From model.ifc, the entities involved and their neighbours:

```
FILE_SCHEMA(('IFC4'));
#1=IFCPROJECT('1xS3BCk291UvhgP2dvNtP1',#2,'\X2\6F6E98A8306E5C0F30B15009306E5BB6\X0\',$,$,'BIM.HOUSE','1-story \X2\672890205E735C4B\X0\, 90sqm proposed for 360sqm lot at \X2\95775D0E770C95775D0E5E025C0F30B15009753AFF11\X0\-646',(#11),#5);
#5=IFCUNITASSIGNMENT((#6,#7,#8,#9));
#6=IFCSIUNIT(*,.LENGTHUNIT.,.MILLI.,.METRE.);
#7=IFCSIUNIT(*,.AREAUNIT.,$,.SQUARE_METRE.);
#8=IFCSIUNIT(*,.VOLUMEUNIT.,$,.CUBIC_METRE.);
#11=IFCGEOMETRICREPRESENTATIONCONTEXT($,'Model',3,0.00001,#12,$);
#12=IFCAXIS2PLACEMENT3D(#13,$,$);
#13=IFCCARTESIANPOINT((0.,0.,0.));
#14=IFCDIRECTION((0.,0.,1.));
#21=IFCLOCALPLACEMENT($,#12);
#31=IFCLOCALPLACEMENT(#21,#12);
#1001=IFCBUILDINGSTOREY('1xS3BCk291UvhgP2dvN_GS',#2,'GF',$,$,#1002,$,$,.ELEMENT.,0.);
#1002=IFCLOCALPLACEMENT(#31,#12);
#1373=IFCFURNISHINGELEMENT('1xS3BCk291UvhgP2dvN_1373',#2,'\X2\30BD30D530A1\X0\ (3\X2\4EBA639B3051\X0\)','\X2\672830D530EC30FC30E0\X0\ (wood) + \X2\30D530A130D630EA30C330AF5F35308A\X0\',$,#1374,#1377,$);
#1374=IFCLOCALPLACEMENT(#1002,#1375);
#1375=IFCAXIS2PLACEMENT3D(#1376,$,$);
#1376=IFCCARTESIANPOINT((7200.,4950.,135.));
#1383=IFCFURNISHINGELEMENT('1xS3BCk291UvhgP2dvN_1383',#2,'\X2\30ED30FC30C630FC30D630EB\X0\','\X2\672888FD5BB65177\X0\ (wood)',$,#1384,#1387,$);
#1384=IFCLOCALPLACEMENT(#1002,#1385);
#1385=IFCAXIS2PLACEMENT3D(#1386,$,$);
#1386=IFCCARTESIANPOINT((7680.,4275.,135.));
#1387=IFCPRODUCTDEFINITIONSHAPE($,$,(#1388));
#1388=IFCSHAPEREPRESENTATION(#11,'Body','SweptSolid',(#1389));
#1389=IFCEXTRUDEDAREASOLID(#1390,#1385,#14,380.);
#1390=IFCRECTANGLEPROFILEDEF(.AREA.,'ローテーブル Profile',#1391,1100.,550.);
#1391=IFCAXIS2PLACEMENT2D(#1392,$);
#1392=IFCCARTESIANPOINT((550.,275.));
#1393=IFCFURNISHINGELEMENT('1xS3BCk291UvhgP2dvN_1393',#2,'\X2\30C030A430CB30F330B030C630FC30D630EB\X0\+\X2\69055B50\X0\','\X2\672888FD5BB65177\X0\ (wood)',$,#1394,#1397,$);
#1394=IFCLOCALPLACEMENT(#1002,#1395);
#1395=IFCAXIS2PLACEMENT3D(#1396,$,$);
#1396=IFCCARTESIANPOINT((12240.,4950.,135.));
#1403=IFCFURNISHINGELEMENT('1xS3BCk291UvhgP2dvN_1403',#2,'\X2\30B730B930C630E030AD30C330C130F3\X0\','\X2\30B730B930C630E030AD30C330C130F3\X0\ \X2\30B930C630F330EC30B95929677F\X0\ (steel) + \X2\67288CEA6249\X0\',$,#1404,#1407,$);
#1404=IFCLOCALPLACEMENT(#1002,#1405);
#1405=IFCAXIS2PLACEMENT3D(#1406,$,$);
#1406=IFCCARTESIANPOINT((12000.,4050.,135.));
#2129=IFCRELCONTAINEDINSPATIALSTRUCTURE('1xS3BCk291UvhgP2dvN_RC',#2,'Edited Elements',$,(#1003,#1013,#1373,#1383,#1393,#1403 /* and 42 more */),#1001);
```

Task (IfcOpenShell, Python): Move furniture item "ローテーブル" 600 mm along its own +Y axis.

```python
import ifcopenshell
import ifcopenshell.api.geometry
import ifcopenshell.util.placement
import ifcopenshell.util.unit

model = ifcopenshell.open("model.ifc")
unit_scale = ifcopenshell.util.unit.calculate_unit_scale(model)

item = model.by_guid("1xS3BCk291UvhgP2dvN_1383")
matrix = ifcopenshell.util.placement.get_local_placement(item.ObjectPlacement)
matrix[:3, 3] += matrix[:3, 1] * 0.6 / unit_scale
ifcopenshell.api.geometry.edit_object_placement(model, product=item, matrix=matrix, is_si=False)

print(ifcopenshell.util.placement.get_local_placement(item.ObjectPlacement).round(3) + 0.0)

model.write("model_v2.ifc")
```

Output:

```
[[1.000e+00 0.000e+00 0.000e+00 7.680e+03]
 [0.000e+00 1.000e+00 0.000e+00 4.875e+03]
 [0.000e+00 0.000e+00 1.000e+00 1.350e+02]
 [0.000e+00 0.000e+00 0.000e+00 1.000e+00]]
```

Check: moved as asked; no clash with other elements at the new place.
